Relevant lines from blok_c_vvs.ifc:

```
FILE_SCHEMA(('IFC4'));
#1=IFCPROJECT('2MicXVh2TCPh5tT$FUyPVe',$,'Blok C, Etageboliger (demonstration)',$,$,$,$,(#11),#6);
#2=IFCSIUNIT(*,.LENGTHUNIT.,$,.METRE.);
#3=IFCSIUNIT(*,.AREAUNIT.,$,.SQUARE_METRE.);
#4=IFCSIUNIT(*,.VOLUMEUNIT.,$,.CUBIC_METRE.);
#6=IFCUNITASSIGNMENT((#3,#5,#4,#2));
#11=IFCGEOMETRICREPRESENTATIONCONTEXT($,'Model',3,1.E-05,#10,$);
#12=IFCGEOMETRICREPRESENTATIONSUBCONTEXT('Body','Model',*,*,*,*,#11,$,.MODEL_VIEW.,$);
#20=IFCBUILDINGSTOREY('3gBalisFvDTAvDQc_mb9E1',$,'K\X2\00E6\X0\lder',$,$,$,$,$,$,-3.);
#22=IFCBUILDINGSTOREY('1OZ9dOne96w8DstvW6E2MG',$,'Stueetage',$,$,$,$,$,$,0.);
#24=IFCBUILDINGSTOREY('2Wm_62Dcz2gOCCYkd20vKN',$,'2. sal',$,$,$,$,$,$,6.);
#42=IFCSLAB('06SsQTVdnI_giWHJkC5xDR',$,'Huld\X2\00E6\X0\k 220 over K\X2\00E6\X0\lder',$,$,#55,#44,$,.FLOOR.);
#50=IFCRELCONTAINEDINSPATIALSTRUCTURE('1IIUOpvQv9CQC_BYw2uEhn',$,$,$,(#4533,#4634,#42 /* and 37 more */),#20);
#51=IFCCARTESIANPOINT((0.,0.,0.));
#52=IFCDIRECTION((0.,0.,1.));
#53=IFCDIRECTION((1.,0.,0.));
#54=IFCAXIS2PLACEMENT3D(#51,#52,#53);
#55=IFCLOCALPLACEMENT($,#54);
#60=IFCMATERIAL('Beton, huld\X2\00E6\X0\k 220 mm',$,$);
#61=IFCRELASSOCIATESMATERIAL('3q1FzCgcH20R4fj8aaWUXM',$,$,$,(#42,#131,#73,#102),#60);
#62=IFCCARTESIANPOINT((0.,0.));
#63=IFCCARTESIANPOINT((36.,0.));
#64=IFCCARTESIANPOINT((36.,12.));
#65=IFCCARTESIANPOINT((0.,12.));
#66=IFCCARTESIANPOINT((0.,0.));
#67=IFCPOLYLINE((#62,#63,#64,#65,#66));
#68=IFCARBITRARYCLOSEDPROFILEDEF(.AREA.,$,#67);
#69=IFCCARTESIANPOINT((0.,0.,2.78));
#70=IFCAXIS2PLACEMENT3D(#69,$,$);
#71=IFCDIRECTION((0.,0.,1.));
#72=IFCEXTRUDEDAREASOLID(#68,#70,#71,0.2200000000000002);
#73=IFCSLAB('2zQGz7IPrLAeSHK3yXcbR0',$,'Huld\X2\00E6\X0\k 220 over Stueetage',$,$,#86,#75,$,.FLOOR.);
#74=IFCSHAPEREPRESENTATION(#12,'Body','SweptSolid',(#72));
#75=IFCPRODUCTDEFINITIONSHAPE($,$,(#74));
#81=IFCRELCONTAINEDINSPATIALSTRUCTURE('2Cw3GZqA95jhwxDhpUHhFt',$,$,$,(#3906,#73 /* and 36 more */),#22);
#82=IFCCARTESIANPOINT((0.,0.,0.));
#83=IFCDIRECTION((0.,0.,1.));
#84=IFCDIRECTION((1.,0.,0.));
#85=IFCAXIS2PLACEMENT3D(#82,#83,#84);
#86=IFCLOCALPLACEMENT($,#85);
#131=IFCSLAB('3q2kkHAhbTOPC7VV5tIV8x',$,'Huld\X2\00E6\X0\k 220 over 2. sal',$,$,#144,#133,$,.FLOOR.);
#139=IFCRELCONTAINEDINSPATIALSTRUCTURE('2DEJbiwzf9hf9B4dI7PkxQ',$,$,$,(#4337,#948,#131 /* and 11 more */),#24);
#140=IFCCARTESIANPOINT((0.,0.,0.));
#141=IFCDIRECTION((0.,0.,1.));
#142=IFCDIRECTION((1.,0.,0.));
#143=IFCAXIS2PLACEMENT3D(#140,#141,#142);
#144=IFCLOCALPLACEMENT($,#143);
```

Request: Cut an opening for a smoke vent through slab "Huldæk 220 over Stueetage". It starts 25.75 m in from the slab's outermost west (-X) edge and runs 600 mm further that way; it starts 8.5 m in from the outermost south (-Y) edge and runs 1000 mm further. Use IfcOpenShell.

```python
import numpy as np
import ifcopenshell
import ifcopenshell.api.feature
import ifcopenshell.api.geometry
import ifcopenshell.api.root
import ifcopenshell.geom
import ifcopenshell.util.placement
import ifcopenshell.util.representation
import ifcopenshell.util.shape
import ifcopenshell.util.unit

model = ifcopenshell.open("blok_c_vvs.ifc")
unit_scale = ifcopenshell.util.unit.calculate_unit_scale(model)
settings = ifcopenshell.geom.settings()


def volume(element):
    """Net volume in cubic metres, openings subtracted."""
    shape = ifcopenshell.geom.create_shape(settings, element)
    return ifcopenshell.util.shape.get_volume(shape.geometry)


slab = model.by_guid("2zQGz7IPrLAeSHK3yXcbR0")
before = volume(slab)

# Extent in the slab's own axes, in metres. The edges named are its -X and -Y sides.
slab_shape = ifcopenshell.geom.create_shape(settings, slab)
vertices = ifcopenshell.util.shape.get_vertices(slab_shape.geometry)
x_min, y_min, bottom = vertices.min(axis=0)
top = vertices[:, 2].max()

opening = ifcopenshell.api.root.create_entity(model, ifc_class="IfcOpeningElement", name="Smoke vent opening", predefined_type="OPENING")
context = ifcopenshell.util.representation.get_context(model, "Model", "Body", "MODEL_VIEW")
width, depth = 0.6, 1
outline = [(0.0, 0.0), (width, 0.0), (width, depth), (0.0, depth), (0.0, 0.0)]
# Overshoot both faces by 50 mm so the cut is clean.
shape = ifcopenshell.api.geometry.add_slab_representation(
    model, context=context, depth=top - bottom + 0.1, polyline=outline
)
ifcopenshell.api.geometry.assign_representation(model, product=opening, representation=shape)

matrix = ifcopenshell.util.placement.get_local_placement(slab.ObjectPlacement)
matrix[:, 3] = matrix @ np.append(np.array([x_min + 25.75, y_min + 8.5, bottom - 0.05]) / unit_scale, 1.0)
ifcopenshell.api.geometry.edit_object_placement(model, product=opening, matrix=matrix, is_si=False)
ifcopenshell.api.feature.add_feature(model, feature=opening, element=slab)

after = volume(slab)

print(f"slab volume {before:.3f} -> {after:.3f} m3")

model.write("blok_c_vvs_rev.ifc")
```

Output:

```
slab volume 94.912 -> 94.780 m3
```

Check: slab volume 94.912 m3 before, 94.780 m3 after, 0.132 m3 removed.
